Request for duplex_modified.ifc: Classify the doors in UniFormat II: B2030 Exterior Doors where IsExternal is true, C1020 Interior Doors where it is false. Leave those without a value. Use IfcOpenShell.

First a look at what the model holds.

```python
import ifcopenshell
import ifcopenshell.util.element

model = ifcopenshell.open("duplex_modified.ifc")
print(model.schema)
print("classifications:", [c.Name for c in model.by_type("IfcClassification")])
values = [ifcopenshell.util.element.get_pset(e, "Pset_DoorCommon", "IsExternal") for e in model.by_type("IfcDoor")]
for value in (True, False, None):
    print("IsExternal", value, values.count(value))
```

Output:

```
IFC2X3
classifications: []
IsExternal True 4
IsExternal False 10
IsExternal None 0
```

```python
import ifcopenshell
import ifcopenshell.api.classification
import ifcopenshell.util.element

model = ifcopenshell.open("duplex_modified.ifc")

# IFC2X3 requires Source and Edition and has no link from the project to the system.
system = model.create_entity("IfcClassification", Source="ASTM", Edition="E1557", Name="UniFormat II")

doors = model.by_type("IfcDoor")
external = {e: ifcopenshell.util.element.get_pset(e, "Pset_DoorCommon", "IsExternal") for e in doors}
for flag, code, name in ((True, "B2030", "Exterior Doors"), (False, "C1020", "Interior Doors")):
    products = [e for e in doors if external[e] is flag]
    ifcopenshell.api.classification.add_reference(
        model, products=products, classification=system, identification=code, name=name
    )
    print(code, len(products))

model.write("duplex_modified-out.ifc")
```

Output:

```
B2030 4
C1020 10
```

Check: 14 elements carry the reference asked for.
